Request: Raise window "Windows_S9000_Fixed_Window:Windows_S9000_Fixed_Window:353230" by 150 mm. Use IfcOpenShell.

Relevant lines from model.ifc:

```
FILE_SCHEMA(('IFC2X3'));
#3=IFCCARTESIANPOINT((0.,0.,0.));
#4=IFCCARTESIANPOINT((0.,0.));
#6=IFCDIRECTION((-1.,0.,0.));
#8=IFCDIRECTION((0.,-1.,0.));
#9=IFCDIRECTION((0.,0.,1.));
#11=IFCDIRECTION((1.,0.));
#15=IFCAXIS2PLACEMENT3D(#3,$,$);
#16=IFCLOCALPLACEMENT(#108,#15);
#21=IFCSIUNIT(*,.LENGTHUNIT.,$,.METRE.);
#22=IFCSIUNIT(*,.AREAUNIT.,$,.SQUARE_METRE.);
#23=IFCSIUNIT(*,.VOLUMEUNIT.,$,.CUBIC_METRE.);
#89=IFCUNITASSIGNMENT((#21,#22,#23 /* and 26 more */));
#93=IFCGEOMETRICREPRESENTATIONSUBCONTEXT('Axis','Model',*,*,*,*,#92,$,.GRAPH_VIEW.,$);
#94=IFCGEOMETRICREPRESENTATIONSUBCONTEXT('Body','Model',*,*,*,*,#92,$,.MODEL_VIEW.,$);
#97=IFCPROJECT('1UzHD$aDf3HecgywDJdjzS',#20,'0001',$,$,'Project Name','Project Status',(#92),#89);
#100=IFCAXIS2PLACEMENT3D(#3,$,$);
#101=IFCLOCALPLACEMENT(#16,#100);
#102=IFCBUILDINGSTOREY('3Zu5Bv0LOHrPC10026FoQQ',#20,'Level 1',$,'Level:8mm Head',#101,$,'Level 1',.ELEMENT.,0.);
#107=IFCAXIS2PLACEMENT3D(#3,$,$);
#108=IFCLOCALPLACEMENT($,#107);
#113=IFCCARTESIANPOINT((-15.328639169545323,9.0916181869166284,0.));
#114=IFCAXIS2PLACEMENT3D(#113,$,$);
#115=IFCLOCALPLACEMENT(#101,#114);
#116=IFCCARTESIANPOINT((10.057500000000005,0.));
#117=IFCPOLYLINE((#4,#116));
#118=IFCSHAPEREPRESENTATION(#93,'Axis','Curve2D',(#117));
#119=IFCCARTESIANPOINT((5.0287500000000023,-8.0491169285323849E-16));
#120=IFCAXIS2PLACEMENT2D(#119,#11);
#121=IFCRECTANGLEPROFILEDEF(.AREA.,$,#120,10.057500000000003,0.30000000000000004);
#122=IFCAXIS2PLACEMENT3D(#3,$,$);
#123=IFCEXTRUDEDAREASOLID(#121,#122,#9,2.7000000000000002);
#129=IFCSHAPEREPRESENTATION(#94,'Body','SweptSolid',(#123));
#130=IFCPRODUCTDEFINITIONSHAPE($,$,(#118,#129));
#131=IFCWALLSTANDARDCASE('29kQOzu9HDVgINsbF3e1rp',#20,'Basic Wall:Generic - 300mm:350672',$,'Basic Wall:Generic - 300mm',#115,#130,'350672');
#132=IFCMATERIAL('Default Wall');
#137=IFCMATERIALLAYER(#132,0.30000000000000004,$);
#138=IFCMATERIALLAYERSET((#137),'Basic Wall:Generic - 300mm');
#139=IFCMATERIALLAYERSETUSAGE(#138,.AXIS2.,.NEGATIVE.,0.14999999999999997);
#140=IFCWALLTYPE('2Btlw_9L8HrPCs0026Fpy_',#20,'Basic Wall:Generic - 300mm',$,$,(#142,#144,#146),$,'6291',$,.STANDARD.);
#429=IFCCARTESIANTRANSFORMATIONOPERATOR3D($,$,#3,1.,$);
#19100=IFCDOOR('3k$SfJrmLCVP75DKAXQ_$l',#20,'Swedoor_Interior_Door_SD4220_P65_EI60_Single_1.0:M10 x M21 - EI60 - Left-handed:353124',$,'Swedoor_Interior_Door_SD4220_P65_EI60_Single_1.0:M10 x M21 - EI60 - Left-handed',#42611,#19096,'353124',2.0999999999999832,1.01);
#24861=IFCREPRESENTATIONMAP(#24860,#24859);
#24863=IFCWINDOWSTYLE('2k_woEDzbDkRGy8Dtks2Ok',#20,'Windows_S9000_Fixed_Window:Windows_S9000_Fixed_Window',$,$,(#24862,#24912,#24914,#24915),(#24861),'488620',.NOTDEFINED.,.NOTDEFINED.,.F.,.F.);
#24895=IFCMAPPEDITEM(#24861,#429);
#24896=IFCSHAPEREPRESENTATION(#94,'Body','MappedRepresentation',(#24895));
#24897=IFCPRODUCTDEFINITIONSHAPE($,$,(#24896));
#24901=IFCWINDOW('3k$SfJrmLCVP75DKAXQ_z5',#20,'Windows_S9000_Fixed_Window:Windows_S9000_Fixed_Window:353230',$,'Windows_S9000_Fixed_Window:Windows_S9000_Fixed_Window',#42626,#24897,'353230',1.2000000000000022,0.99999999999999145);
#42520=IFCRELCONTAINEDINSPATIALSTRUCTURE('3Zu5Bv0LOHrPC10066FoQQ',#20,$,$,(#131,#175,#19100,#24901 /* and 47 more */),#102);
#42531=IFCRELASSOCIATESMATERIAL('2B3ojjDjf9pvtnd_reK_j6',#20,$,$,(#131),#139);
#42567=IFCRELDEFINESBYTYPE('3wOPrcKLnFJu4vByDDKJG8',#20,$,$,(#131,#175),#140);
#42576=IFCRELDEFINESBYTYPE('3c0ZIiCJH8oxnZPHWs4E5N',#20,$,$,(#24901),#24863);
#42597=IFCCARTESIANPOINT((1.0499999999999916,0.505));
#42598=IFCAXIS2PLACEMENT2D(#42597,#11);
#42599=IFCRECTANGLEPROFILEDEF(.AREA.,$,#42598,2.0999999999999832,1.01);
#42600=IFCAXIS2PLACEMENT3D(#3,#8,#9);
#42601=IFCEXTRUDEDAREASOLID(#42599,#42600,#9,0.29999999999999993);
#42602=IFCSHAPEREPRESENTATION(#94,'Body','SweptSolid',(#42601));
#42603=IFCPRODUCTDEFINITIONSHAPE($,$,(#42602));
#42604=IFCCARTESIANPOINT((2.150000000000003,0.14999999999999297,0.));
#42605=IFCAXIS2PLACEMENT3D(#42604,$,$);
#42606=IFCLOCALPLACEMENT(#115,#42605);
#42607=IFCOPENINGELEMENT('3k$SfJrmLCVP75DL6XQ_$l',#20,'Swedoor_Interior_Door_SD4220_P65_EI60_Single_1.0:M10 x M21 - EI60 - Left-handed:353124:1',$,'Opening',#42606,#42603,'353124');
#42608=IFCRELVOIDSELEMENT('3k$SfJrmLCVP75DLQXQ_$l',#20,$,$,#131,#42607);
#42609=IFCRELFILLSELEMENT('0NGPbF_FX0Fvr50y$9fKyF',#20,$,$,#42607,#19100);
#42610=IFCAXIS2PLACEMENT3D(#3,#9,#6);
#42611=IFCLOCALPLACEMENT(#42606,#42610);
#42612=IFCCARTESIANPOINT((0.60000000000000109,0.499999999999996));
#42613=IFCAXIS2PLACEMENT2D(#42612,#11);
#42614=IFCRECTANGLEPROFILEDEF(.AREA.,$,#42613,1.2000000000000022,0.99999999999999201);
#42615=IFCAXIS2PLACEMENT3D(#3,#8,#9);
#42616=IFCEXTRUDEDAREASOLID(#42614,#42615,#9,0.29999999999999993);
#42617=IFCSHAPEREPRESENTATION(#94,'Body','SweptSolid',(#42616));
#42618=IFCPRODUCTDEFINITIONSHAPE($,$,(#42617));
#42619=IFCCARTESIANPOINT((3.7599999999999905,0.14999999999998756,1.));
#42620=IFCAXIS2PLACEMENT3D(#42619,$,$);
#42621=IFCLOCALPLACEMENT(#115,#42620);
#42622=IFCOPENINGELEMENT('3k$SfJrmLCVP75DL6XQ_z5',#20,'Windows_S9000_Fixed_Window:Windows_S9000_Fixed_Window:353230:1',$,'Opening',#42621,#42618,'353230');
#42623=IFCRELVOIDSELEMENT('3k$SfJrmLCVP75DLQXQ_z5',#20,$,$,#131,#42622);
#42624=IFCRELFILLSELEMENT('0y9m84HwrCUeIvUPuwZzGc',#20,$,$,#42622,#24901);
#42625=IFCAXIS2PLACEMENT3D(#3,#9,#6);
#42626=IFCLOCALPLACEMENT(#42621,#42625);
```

```python
import numpy as np
import ifcopenshell
import ifcopenshell.api.geometry
import ifcopenshell.util.placement
import ifcopenshell.util.unit

model = ifcopenshell.open("model.ifc")
unit_scale = ifcopenshell.util.unit.calculate_unit_scale(model)

window = model.by_guid("3k$SfJrmLCVP75DKAXQ_z5")
opening = window.FillsVoids[0].RelatingOpeningElement
dz = 0.15 / unit_scale

shift = np.array([0.0, 0.0, dz])
# The window is placed relative to its opening, so it follows when the opening moves.
matrix = ifcopenshell.util.placement.get_local_placement(opening.ObjectPlacement)
matrix[:3, 3] += shift
ifcopenshell.api.geometry.edit_object_placement(
    model, product=opening, matrix=matrix, is_si=False, should_transform_children=True
)

print(f"moved by {dz * unit_scale:+.3f} m")

model.write("model_updated.ifc")
```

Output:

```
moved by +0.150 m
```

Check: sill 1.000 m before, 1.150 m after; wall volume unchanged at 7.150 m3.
